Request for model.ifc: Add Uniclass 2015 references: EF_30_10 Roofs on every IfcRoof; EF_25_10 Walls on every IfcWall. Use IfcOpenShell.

First a look at what the model holds.

```python
import ifcopenshell

model = ifcopenshell.open("model.ifc")
print(model.schema)
print("classifications:", [c.Name for c in model.by_type("IfcClassification")])
for ifc_class in ("IfcDoor", "IfcRoof", "IfcStair", "IfcWall", "IfcWindow"):
    print(ifc_class, len(model.by_type(ifc_class)))
```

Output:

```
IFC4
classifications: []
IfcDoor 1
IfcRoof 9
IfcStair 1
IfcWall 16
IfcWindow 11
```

```python
import ifcopenshell
import ifcopenshell.api.classification

model = ifcopenshell.open("model.ifc")

system = ifcopenshell.api.classification.add_classification(model, classification="Uniclass 2015")

codes = {
    "IfcRoof": ("EF_30_10", "Roofs"),
    "IfcWall": ("EF_25_10", "Walls"),
}
for ifc_class, (code, name) in codes.items():
    products = model.by_type(ifc_class)
    ifcopenshell.api.classification.add_reference(
        model, products=products, classification=system, identification=code, name=name
    )
    print(code, len(products))

model.write("model_rev.ifc")
```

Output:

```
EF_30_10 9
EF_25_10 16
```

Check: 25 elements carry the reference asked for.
